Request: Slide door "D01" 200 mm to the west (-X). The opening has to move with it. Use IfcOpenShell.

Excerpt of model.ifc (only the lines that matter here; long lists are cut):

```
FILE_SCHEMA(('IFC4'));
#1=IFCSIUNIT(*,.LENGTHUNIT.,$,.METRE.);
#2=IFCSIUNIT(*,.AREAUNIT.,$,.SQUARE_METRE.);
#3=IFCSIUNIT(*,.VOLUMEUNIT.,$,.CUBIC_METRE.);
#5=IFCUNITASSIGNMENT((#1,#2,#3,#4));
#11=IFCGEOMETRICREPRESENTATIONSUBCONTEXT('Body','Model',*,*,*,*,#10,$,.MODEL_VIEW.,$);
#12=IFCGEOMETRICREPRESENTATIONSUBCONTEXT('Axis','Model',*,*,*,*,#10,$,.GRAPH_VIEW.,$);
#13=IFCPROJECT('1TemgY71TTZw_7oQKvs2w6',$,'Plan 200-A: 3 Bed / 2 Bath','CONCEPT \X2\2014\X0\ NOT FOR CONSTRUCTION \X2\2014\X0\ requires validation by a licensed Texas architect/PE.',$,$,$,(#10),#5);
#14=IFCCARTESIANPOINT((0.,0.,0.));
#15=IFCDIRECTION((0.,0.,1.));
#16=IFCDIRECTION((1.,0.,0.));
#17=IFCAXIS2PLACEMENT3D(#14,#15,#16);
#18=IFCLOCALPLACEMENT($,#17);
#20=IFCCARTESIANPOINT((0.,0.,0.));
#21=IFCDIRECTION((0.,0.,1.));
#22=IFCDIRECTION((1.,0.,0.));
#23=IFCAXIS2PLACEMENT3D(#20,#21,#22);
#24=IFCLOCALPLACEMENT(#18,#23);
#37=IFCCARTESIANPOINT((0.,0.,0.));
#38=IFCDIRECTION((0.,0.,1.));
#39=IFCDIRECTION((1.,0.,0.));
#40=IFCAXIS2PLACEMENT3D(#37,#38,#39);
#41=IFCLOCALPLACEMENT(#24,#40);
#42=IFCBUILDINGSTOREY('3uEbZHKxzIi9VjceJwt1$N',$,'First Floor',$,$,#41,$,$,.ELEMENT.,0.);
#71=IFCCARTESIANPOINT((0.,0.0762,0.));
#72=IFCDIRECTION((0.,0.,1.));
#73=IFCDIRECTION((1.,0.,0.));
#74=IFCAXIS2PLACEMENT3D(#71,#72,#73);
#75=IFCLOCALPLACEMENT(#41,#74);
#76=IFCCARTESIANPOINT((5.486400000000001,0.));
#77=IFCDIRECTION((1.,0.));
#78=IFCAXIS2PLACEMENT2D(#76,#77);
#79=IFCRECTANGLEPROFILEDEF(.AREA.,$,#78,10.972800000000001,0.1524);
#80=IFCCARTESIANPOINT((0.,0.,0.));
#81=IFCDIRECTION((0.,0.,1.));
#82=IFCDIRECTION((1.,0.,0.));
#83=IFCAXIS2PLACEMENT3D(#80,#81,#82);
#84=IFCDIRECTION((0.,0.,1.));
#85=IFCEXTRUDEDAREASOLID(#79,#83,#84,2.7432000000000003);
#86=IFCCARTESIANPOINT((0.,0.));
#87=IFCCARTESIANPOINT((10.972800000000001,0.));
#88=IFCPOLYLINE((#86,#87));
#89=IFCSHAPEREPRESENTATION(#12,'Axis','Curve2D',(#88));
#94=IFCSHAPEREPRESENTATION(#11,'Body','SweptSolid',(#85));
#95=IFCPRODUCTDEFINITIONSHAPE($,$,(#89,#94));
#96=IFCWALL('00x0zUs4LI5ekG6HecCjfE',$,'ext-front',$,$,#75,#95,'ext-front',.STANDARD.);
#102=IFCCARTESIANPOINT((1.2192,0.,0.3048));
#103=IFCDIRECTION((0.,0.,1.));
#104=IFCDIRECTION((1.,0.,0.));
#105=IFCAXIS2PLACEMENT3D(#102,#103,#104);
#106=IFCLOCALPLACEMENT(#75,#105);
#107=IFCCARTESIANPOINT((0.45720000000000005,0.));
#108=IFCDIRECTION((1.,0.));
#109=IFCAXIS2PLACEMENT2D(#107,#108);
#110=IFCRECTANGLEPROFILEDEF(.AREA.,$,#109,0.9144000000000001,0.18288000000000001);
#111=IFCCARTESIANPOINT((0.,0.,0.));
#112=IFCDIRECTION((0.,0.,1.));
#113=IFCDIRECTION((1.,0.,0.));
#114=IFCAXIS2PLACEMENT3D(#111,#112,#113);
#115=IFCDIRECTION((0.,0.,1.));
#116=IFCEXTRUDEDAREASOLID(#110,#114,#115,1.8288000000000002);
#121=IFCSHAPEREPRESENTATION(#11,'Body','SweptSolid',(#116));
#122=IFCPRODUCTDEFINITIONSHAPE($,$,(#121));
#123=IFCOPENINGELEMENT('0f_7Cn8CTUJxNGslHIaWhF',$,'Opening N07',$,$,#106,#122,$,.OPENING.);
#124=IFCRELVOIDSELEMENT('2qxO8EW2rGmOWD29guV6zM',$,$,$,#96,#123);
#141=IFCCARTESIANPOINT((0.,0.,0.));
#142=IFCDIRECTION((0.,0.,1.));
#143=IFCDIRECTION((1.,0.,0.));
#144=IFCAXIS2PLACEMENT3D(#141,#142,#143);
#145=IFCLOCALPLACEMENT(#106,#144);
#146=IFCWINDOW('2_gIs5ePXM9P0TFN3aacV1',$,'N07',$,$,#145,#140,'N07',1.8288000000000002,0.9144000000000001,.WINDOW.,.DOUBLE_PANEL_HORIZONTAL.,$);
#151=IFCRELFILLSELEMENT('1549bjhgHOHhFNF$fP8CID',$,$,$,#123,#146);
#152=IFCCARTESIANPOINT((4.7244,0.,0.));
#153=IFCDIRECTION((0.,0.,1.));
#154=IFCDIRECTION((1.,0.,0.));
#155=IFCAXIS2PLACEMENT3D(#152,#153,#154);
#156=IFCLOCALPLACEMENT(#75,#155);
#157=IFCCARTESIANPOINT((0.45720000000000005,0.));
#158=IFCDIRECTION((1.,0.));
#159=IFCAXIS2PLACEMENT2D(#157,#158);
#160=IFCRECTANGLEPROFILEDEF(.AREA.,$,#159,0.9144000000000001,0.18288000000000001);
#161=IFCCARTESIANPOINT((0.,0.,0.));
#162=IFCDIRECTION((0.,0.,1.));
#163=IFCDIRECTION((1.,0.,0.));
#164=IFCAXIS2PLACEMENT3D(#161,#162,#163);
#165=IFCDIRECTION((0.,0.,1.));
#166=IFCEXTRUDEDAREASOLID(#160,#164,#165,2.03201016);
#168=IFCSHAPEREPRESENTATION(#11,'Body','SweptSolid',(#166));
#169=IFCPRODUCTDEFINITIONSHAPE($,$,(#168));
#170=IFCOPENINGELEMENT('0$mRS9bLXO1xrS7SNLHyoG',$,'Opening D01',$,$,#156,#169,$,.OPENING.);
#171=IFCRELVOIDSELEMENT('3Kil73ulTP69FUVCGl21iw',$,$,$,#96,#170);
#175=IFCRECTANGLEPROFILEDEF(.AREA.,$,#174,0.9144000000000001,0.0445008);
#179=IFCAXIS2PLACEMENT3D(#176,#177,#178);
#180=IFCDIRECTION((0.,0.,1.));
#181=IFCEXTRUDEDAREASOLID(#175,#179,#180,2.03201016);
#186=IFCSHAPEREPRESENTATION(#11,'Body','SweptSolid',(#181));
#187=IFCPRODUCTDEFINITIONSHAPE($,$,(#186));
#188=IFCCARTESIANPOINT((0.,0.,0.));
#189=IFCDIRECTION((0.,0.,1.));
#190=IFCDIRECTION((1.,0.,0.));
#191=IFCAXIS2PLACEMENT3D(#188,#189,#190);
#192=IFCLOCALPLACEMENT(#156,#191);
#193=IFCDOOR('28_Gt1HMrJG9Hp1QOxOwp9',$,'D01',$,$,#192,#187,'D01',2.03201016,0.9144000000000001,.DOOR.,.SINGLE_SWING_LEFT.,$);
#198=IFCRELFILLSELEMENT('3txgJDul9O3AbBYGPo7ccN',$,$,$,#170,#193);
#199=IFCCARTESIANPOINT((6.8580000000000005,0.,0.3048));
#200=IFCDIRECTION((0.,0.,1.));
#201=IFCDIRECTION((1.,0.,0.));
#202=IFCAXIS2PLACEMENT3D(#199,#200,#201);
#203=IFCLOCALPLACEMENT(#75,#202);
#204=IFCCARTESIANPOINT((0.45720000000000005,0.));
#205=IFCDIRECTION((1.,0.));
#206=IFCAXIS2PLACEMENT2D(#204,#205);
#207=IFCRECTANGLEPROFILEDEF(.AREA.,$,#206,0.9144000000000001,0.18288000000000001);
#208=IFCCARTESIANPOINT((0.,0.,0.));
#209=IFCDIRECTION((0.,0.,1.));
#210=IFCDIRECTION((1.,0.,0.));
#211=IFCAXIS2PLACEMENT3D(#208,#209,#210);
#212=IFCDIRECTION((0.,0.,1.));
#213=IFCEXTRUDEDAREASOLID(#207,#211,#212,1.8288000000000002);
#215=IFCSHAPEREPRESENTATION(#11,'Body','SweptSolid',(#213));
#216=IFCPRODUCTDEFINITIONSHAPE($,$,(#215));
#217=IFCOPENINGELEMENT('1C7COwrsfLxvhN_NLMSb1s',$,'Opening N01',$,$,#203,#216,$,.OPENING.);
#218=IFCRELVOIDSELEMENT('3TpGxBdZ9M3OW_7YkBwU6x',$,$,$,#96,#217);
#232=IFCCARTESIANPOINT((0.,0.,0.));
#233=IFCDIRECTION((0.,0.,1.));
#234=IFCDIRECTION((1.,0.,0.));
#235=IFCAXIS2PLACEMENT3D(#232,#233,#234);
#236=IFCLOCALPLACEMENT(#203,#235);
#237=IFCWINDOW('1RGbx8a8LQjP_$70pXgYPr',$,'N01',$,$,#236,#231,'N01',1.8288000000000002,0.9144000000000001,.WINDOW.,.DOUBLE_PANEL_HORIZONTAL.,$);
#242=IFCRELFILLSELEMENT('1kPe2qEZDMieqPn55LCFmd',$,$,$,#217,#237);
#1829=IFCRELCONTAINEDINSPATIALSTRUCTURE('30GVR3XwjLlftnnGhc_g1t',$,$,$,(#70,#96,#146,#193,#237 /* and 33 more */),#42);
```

```python
import ifcopenshell
import ifcopenshell.api.geometry
import ifcopenshell.util.placement

model = ifcopenshell.open("model.ifc")

door = model.by_guid("28_Gt1HMrJG9Hp1QOxOwp9")
opening = door.FillsVoids[0].RelatingOpeningElement
wall = opening.VoidsElements[0].RelatingBuildingElement

wall_matrix = ifcopenshell.util.placement.get_local_placement(wall.ObjectPlacement)
shift = wall_matrix[:3, 0] * -0.2
before = ifcopenshell.util.placement.get_local_placement(door.ObjectPlacement)[:3, 3].copy()

# The door is placed relative to its opening, so it follows when the opening moves.
matrix = ifcopenshell.util.placement.get_local_placement(opening.ObjectPlacement)
matrix[:3, 3] += shift
ifcopenshell.api.geometry.edit_object_placement(
    model, product=opening, matrix=matrix, is_si=False, should_transform_children=True
)

after = ifcopenshell.util.placement.get_local_placement(door.ObjectPlacement)[:3, 3]
print("door moved by", (after - before).round(3) + 0.0)

model.write("model_edited.ifc")
```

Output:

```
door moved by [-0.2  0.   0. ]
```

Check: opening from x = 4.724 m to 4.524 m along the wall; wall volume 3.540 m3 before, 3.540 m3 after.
